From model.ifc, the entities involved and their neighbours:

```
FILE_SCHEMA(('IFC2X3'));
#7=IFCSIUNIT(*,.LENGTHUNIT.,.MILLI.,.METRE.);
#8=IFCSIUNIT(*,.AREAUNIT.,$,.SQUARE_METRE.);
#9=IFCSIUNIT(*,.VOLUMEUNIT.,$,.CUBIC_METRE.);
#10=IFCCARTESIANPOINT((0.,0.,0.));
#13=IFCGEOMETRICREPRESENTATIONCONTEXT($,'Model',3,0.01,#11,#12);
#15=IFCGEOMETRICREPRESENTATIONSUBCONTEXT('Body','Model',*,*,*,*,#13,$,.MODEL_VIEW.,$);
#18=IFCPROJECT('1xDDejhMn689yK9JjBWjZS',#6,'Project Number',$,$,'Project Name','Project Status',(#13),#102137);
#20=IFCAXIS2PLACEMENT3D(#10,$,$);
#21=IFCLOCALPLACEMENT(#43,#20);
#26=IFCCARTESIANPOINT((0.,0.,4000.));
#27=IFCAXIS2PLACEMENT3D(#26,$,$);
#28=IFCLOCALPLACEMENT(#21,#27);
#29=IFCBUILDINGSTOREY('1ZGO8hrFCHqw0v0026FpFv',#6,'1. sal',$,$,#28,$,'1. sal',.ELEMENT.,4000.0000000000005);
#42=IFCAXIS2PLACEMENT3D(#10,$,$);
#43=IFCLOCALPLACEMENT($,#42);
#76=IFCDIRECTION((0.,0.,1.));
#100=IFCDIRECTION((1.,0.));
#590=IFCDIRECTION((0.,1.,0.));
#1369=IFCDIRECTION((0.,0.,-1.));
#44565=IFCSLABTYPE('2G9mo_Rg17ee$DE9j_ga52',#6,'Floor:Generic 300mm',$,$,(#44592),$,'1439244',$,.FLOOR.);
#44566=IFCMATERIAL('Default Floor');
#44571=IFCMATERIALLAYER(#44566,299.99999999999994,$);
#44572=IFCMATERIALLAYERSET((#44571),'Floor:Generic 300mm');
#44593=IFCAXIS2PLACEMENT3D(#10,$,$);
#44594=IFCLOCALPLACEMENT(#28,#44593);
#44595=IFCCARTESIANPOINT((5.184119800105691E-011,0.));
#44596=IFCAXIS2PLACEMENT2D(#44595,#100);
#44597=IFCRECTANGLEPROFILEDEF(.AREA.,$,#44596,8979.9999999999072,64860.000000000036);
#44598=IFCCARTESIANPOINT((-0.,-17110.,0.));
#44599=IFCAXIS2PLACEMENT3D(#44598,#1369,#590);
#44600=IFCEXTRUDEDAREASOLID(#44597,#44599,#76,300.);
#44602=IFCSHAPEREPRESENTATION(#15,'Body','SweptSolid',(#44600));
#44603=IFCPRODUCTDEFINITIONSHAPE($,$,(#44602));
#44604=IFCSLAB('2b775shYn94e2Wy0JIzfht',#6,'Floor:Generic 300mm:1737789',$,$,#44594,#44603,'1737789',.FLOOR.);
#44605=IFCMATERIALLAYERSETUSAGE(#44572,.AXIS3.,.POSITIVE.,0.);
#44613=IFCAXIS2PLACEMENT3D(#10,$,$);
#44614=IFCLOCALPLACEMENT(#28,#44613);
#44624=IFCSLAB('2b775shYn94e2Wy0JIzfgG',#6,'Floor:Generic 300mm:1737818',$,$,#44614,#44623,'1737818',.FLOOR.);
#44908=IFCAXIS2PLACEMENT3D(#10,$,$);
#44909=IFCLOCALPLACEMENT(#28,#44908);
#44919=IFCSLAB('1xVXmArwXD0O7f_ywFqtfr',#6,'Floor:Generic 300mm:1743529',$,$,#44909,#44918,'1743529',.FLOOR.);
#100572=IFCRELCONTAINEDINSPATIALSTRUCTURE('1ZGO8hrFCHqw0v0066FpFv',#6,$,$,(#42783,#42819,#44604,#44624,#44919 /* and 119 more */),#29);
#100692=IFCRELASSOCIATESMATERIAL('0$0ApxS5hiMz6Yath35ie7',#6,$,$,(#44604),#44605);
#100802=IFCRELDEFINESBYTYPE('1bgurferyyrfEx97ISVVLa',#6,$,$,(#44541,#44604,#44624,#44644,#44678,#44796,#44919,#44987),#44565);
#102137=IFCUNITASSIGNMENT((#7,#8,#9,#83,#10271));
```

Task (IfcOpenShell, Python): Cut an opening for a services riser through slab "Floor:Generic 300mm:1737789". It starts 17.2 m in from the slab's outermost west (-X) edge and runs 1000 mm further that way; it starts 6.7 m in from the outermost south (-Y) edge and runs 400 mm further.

```python
import numpy as np
import ifcopenshell
import ifcopenshell.api.feature
import ifcopenshell.api.geometry
import ifcopenshell.api.root
import ifcopenshell.geom
import ifcopenshell.util.placement
import ifcopenshell.util.representation
import ifcopenshell.util.shape
import ifcopenshell.util.unit

model = ifcopenshell.open("model.ifc")
unit_scale = ifcopenshell.util.unit.calculate_unit_scale(model)
settings = ifcopenshell.geom.settings()


def volume(element):
    """Net volume in cubic metres, openings subtracted."""
    shape = ifcopenshell.geom.create_shape(settings, element)
    return ifcopenshell.util.shape.get_volume(shape.geometry)


slab = model.by_guid("2b775shYn94e2Wy0JIzfht")
before = volume(slab)

# Extent in the slab's own axes, in metres. The edges named are its -X and -Y sides.
slab_shape = ifcopenshell.geom.create_shape(settings, slab)
vertices = ifcopenshell.util.shape.get_vertices(slab_shape.geometry)
x_min, y_min, bottom = vertices.min(axis=0)
top = vertices[:, 2].max()

opening = ifcopenshell.api.root.create_entity(model, ifc_class="IfcOpeningElement", name="Services riser opening")
context = ifcopenshell.util.representation.get_context(model, "Model", "Body", "MODEL_VIEW")
width, depth = 1, 0.4
outline = [(0.0, 0.0), (width, 0.0), (width, depth), (0.0, depth), (0.0, 0.0)]
# Overshoot both faces by 50 mm so the cut is clean.
shape = ifcopenshell.api.geometry.add_slab_representation(
    model, context=context, depth=top - bottom + 0.1, polyline=outline
)
ifcopenshell.api.geometry.assign_representation(model, product=opening, representation=shape)

matrix = ifcopenshell.util.placement.get_local_placement(slab.ObjectPlacement)
matrix[:, 3] = matrix @ np.append(np.array([x_min + 17.2, y_min + 6.7, bottom - 0.05]) / unit_scale, 1.0)
ifcopenshell.api.geometry.edit_object_placement(model, product=opening, matrix=matrix, is_si=False)
ifcopenshell.api.feature.add_feature(model, feature=opening, element=slab)

after = volume(slab)

print(f"slab volume {before:.3f} -> {after:.3f} m3")

model.write("model_updated.ifc")
```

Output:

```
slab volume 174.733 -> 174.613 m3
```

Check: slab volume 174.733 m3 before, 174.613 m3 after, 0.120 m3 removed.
